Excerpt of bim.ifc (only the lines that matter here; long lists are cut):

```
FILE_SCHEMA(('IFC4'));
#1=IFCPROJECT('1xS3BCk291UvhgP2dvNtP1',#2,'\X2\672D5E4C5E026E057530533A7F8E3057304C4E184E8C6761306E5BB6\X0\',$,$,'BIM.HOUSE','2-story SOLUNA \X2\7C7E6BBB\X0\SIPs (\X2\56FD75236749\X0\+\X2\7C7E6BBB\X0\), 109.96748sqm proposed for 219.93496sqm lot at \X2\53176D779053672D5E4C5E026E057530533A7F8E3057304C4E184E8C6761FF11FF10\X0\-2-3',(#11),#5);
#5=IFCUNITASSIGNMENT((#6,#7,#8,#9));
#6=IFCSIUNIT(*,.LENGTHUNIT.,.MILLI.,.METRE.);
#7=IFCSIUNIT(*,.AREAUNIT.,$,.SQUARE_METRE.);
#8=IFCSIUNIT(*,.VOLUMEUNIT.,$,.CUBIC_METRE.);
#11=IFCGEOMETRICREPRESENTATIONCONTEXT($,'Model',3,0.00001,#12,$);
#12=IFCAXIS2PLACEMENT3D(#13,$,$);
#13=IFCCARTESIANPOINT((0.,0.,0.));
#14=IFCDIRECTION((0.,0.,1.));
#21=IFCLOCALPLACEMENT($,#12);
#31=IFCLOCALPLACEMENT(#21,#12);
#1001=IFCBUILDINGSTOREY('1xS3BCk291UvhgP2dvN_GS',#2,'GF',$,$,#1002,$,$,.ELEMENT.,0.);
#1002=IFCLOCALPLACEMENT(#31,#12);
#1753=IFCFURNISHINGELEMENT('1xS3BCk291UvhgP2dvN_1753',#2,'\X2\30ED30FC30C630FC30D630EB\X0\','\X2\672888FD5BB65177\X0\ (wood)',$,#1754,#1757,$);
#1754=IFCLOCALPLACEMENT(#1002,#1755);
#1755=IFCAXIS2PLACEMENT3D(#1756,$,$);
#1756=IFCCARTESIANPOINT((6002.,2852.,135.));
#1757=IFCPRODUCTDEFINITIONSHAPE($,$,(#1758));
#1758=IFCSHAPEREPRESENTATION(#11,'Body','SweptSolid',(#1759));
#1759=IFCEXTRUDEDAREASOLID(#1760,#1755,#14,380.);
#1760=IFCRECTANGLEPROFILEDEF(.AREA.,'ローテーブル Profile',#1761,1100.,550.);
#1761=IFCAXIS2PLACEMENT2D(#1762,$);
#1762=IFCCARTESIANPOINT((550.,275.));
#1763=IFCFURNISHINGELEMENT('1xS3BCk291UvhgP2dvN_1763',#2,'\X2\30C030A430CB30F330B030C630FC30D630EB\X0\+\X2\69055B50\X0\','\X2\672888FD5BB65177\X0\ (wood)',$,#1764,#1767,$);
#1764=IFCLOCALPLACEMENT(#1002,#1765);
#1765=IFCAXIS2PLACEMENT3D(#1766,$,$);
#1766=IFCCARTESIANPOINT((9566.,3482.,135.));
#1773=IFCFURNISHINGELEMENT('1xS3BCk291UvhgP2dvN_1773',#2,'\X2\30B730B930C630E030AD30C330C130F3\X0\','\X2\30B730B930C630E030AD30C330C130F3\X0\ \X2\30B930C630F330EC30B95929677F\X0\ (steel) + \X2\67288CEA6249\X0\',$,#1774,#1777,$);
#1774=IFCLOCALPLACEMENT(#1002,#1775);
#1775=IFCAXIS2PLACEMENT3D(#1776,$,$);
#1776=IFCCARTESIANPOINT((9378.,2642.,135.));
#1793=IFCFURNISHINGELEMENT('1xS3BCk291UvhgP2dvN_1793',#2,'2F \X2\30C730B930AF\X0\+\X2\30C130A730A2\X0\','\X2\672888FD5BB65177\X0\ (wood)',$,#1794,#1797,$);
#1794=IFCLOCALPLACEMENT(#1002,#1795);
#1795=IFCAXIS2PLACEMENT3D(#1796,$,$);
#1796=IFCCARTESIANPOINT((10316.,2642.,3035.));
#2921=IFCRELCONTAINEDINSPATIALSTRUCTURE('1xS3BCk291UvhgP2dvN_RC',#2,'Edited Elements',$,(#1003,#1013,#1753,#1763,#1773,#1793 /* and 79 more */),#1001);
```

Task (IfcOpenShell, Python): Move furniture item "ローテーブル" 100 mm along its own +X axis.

```python
import ifcopenshell
import ifcopenshell.api.geometry
import ifcopenshell.util.placement
import ifcopenshell.util.unit

model = ifcopenshell.open("bim.ifc")
unit_scale = ifcopenshell.util.unit.calculate_unit_scale(model)

item = model.by_guid("1xS3BCk291UvhgP2dvN_1753")
matrix = ifcopenshell.util.placement.get_local_placement(item.ObjectPlacement)
matrix[:3, 3] += matrix[:3, 0] * 0.1 / unit_scale
ifcopenshell.api.geometry.edit_object_placement(model, product=item, matrix=matrix, is_si=False)

print(ifcopenshell.util.placement.get_local_placement(item.ObjectPlacement).round(3) + 0.0)

model.write("bim_edited.ifc")
```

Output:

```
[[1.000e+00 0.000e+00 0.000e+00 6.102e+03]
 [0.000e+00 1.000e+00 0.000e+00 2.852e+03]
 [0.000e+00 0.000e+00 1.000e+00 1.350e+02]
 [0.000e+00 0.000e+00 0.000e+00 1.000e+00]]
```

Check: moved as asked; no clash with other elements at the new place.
